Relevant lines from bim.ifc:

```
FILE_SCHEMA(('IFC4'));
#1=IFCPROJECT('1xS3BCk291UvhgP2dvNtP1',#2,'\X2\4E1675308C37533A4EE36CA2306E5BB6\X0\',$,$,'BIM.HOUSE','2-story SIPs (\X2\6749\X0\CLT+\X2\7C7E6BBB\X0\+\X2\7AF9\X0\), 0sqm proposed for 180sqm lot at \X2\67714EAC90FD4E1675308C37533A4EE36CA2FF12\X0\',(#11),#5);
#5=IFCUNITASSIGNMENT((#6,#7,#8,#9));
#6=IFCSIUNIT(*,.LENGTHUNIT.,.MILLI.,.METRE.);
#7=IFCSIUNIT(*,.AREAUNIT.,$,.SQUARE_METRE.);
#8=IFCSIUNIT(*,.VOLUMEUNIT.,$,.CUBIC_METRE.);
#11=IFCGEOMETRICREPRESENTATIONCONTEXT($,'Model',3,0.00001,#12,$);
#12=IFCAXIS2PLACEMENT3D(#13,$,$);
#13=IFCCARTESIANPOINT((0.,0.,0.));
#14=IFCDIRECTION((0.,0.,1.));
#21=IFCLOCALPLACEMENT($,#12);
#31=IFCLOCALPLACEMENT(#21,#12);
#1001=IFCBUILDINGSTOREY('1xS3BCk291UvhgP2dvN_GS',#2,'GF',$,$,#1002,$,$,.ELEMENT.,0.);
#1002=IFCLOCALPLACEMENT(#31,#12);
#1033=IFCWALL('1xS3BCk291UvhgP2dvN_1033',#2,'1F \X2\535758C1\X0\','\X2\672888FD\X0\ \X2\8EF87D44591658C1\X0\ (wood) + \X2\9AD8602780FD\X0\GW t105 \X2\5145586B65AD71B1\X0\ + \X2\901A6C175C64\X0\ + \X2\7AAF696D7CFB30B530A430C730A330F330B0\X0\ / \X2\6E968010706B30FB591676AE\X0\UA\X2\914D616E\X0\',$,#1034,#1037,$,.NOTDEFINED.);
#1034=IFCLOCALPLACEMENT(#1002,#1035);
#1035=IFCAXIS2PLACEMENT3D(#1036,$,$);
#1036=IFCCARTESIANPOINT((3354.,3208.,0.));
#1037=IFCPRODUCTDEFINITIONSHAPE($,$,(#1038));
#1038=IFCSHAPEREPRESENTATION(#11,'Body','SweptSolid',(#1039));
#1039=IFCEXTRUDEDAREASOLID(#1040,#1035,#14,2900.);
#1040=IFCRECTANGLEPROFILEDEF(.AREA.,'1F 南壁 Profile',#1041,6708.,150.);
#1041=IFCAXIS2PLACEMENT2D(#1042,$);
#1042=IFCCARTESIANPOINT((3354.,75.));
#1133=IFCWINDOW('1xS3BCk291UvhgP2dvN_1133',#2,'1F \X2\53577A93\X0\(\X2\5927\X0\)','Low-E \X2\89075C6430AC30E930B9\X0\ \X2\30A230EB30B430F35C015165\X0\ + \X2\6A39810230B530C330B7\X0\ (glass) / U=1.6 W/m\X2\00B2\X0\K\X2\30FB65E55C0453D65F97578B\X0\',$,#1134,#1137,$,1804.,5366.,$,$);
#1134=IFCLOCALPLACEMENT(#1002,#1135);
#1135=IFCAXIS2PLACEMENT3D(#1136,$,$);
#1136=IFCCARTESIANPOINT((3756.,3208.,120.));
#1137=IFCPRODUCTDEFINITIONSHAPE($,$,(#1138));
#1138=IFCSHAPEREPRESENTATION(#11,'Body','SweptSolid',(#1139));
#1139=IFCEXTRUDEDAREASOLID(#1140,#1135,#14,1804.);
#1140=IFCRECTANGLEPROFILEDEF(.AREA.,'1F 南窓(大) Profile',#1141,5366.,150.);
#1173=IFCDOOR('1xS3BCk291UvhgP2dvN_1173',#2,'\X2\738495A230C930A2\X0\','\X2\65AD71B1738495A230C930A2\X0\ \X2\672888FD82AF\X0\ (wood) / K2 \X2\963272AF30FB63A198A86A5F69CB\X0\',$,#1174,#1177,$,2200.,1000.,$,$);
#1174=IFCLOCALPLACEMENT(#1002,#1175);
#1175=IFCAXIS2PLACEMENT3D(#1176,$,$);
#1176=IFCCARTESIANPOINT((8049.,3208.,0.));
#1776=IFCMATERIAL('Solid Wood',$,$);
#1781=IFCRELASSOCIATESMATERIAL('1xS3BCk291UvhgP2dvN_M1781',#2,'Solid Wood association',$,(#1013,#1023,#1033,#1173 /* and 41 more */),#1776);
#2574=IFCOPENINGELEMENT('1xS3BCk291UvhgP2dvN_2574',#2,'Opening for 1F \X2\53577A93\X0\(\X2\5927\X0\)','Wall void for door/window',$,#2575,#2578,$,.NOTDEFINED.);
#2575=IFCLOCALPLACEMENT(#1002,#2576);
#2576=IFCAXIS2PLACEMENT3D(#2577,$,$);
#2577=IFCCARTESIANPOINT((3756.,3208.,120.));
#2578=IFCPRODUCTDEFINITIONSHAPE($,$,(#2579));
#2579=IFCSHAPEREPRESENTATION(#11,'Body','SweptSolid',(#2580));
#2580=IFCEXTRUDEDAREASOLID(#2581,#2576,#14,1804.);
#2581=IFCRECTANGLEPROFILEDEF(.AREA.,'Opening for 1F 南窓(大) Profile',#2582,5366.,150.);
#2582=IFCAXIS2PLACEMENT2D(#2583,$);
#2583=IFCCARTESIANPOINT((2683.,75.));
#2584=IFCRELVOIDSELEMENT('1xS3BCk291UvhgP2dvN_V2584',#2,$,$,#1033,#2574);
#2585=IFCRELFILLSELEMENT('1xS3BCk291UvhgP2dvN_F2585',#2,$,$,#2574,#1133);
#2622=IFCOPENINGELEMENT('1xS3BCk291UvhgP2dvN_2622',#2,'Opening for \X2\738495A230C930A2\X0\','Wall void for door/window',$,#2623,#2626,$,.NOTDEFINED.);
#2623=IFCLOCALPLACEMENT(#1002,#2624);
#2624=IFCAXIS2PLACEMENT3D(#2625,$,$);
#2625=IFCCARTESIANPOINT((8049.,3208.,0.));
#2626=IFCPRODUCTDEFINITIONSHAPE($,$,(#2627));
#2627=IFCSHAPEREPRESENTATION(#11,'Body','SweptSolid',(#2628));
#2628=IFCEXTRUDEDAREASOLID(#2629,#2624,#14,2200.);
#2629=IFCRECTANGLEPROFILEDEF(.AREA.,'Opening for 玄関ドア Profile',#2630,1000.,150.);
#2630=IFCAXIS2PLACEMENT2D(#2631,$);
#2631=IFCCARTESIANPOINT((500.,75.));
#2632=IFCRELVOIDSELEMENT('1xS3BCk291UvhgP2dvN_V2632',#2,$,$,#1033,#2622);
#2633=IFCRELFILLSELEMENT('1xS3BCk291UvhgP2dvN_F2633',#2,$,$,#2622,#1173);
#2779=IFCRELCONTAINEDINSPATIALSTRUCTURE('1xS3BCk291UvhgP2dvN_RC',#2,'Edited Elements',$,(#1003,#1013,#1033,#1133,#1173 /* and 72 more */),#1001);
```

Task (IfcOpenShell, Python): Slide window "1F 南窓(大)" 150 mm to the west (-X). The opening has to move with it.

```python
import ifcopenshell
import ifcopenshell.api.geometry
import ifcopenshell.util.placement

model = ifcopenshell.open("bim.ifc")

window = model.by_id(1133)
opening = window.FillsVoids[0].RelatingOpeningElement
wall = opening.VoidsElements[0].RelatingBuildingElement

wall_matrix = ifcopenshell.util.placement.get_local_placement(wall.ObjectPlacement)
shift = wall_matrix[:3, 0] * -150.0
before = ifcopenshell.util.placement.get_local_placement(window.ObjectPlacement)[:3, 3].copy()

# The window is not placed relative to its opening, so move both.
for product in (opening, window):
    matrix = ifcopenshell.util.placement.get_local_placement(product.ObjectPlacement)
    matrix[:3, 3] += shift
    ifcopenshell.api.geometry.edit_object_placement(model, product=product, matrix=matrix, is_si=False)

after = ifcopenshell.util.placement.get_local_placement(window.ObjectPlacement)[:3, 3]
print("window moved by", (after - before).round(3) + 0.0)

model.write("bim_v2.ifc")
```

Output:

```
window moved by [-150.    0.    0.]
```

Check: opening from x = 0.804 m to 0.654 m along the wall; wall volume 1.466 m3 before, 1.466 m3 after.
